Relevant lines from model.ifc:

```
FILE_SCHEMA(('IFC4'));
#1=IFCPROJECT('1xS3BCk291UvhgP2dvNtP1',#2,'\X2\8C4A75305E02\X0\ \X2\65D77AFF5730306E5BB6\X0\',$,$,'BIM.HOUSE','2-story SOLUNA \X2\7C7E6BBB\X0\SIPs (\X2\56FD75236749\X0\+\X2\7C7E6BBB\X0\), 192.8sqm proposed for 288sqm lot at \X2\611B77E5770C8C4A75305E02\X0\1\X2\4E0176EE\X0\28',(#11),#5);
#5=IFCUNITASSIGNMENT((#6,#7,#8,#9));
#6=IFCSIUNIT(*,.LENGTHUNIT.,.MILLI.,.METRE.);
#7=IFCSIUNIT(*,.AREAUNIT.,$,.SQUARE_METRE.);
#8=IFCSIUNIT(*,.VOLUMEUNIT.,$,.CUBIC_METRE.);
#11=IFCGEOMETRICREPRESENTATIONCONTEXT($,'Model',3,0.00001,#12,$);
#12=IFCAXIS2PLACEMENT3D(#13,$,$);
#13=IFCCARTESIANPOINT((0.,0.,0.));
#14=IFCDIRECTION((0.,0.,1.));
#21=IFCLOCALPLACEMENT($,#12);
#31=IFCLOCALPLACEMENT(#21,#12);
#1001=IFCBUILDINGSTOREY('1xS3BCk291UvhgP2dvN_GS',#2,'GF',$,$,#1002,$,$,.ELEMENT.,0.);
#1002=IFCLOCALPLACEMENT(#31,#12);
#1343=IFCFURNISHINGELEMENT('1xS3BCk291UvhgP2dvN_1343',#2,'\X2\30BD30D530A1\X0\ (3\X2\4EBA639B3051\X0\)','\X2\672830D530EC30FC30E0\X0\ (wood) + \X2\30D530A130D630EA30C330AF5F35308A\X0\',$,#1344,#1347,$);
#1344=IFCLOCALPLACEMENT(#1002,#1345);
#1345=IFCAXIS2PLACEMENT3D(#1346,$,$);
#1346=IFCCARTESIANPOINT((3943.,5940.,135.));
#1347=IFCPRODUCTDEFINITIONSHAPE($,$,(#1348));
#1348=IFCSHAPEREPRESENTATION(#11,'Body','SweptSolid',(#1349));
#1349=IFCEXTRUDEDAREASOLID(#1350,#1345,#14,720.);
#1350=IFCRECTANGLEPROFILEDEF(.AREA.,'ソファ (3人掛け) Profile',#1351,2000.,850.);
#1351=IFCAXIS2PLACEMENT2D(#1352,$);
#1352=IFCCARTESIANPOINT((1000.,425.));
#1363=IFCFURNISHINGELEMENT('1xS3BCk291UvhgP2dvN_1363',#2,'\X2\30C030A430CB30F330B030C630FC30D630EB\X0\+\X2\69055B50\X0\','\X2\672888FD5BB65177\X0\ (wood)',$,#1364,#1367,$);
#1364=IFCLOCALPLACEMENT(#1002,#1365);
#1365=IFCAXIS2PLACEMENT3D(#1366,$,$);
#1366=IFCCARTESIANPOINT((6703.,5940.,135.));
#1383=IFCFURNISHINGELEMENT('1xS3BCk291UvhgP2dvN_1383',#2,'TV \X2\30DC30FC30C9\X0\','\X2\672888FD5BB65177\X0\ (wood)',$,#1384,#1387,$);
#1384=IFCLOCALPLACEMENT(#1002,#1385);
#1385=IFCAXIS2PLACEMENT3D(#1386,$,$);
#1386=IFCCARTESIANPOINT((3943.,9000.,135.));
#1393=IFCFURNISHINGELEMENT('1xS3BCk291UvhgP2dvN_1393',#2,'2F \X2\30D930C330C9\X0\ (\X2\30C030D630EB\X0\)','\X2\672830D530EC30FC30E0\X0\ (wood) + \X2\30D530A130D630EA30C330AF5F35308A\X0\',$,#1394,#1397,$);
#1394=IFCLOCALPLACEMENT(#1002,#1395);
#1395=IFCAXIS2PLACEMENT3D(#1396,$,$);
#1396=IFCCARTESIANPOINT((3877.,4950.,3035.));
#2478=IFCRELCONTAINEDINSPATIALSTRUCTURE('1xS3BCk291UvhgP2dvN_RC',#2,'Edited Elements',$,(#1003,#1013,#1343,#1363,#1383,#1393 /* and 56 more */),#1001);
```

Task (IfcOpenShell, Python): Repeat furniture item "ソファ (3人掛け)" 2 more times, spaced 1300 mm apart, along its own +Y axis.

```python
import ifcopenshell
import ifcopenshell.api.geometry
import ifcopenshell.api.root
import ifcopenshell.util.element
import ifcopenshell.util.placement
import ifcopenshell.util.unit

model = ifcopenshell.open("model.ifc")
unit_scale = ifcopenshell.util.unit.calculate_unit_scale(model)


def reuse_history(source, copy):
    """copy_class also copies each property set's owner history, people and application; keep the originals."""
    for rel in copy.IsDefinedBy:
        if rel.is_a("IfcRelDefinesByProperties") and (history := rel.RelatingPropertyDefinition.OwnerHistory):
            rel.RelatingPropertyDefinition.OwnerHistory = source.OwnerHistory
            ifcopenshell.util.element.remove_deep2(model, history)


source = model.by_guid("1xS3BCk291UvhgP2dvN_1343")
base = ifcopenshell.util.placement.get_local_placement(source.ObjectPlacement)
step = base[:3, 1] * 1.3 / unit_scale

for i in range(1, 3):
    copy = ifcopenshell.api.root.copy_class(model, product=source)
    copy.Representation = ifcopenshell.util.element.copy_deep(
        model, source.Representation, exclude=["IfcGeometricRepresentationContext", "IfcRepresentationMap"]
    )
    reuse_history(source, copy)
    matrix = base.copy()
    matrix[:3, 3] += i * step
    print("added at", matrix[:3, 3].round(3) + 0.0)
    ifcopenshell.api.geometry.edit_object_placement(model, product=copy, matrix=matrix, is_si=False)

model.write("model_updated.ifc")
```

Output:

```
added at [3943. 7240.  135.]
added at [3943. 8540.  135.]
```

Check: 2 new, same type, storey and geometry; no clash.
